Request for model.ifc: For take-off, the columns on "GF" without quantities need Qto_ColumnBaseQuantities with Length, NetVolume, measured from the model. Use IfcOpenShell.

First a look at what the model holds.

```python
import ifcopenshell
import ifcopenshell.util.element
import ifcopenshell.util.unit

model = ifcopenshell.open("model.ifc")
print(model.schema)
for unit_type in ("LENGTHUNIT", "AREAUNIT", "VOLUMEUNIT"):
    print(unit_type, ifcopenshell.util.unit.calculate_unit_scale(model, unit_type))
storey = next(s for s in model.by_type("IfcBuildingStorey") if s.Name == "GF")
columns = [e for e in ifcopenshell.util.element.get_decomposition(storey) if e.is_a("IfcColumn")]
for e in sorted(columns, key=lambda e: e.id()):
    print(e.id(), e.is_a(), e.Name, list(ifcopenshell.util.element.get_psets(e, qtos_only=True)), sep=" | ")
```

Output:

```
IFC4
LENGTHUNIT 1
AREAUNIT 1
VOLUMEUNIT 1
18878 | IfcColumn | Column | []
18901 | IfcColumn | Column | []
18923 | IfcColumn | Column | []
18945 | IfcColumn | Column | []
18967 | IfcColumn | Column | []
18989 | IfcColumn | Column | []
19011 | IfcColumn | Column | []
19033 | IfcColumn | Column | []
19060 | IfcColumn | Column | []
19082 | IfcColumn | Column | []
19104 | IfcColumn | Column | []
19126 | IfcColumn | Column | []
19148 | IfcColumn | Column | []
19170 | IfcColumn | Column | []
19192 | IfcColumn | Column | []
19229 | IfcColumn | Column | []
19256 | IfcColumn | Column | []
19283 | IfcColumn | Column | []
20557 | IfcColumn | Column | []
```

```python
import ifcopenshell
import ifcopenshell.api.pset
import ifcopenshell.geom
import ifcopenshell.util.element
import ifcopenshell.util.shape
import ifcopenshell.util.unit

model = ifcopenshell.open("model.ifc")
unit_scale = ifcopenshell.util.unit.calculate_unit_scale(model)
volume_scale = ifcopenshell.util.unit.calculate_unit_scale(model, "VOLUMEUNIT")
settings = ifcopenshell.geom.settings()

storey = next(s for s in model.by_type("IfcBuildingStorey") if s.Name == "GF")
columns = [e for e in ifcopenshell.util.element.get_decomposition(storey) if e.is_a("IfcColumn")]

for e in sorted(columns, key=lambda e: e.id()):
    if ifcopenshell.util.element.get_psets(e, qtos_only=True, should_inherit=False):
        continue
    # Geometry comes back in metres, in the element's own axes.
    shape = ifcopenshell.geom.create_shape(settings, e)
    values = {
        "Length": ifcopenshell.util.shape.get_z(shape.geometry) / unit_scale,
        "NetVolume": ifcopenshell.util.shape.get_volume(shape.geometry) / volume_scale,
    }
    qto = ifcopenshell.api.pset.add_qto(model, product=e, name="Qto_ColumnBaseQuantities")
    ifcopenshell.api.pset.edit_qto(model, qto=qto, properties=values)
    print(e.id(), {k: round(v, 3) for k, v in values.items()})

model.write("model_rev.ifc")
```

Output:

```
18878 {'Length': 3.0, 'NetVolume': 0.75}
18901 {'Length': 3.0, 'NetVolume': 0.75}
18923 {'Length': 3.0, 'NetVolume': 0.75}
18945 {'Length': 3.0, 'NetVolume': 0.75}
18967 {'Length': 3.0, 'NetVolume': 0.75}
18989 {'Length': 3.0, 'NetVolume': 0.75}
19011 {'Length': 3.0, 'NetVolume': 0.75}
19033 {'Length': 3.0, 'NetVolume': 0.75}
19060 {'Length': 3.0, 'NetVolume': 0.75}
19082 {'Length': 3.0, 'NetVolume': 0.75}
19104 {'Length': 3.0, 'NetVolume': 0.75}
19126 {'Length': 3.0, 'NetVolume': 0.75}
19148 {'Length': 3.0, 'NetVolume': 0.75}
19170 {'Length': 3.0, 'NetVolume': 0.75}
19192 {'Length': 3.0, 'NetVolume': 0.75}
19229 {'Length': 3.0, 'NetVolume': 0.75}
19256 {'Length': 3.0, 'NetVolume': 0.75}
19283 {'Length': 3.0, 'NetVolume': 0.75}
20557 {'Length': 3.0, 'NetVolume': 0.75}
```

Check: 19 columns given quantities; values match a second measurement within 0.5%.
